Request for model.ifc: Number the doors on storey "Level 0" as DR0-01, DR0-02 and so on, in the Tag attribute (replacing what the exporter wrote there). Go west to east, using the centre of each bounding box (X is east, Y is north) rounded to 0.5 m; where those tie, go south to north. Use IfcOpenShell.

First a look at what the model holds.

```python
import ifcopenshell
import ifcopenshell.util.element
import ifcopenshell.util.placement

model = ifcopenshell.open("model.ifc")
print(model.schema)
storey = next(s for s in model.by_type("IfcBuildingStorey") if s.Name == "Level 0")
doors = [e for e in ifcopenshell.util.element.get_decomposition(storey) if e.is_a("IfcDoor")]
for e in sorted(doors, key=lambda e: e.id()):
    origin = ifcopenshell.util.placement.get_local_placement(e.ObjectPlacement)[:3, 3]
    print(e.id(), e.Tag, e.Name, origin.round(2) + 0.0, sep=" | ")
```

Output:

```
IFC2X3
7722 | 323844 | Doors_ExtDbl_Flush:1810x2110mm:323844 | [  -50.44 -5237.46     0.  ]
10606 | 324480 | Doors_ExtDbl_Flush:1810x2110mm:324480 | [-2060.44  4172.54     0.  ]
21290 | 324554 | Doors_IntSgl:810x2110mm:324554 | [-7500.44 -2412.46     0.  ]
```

```python
import ifcopenshell
import ifcopenshell.geom
import ifcopenshell.util.element
import ifcopenshell.util.shape

model = ifcopenshell.open("model.ifc")
settings = ifcopenshell.geom.settings()
settings.set("use-world-coords", True)


def centre(element):
    shape = ifcopenshell.geom.create_shape(settings, element)
    return ifcopenshell.util.shape.get_bbox_centroid(shape.geometry)


storey = next(s for s in model.by_type("IfcBuildingStorey") if s.Name == "Level 0")
doors = [e for e in ifcopenshell.util.element.get_decomposition(storey) if e.is_a("IfcDoor")]

# Insertion points can sit at a corner or the storey origin, so sort by the geometry (in metres).
centres = {e: centre(e) for e in doors}
doors.sort(key=lambda e: (round(centres[e][0] / 0.5), centres[e][1]))

for i, e in enumerate(doors, start=1):
    number = f"DR0-{i:02d}"
    e.Tag = number
    print(e.id(), number)

model.write("model_v2.ifc")
```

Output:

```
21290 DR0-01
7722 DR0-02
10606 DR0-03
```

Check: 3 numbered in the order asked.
